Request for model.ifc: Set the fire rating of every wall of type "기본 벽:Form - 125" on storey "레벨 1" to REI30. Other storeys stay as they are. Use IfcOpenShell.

First a look at what the model holds.

```python
import ifcopenshell
import ifcopenshell.util.element

model = ifcopenshell.open("model.ifc")
print(model.schema)
storey = next(s for s in model.by_type("IfcBuildingStorey") if s.Name == "레벨 1")
walls = [e for e in ifcopenshell.util.element.get_decomposition(storey) if e.is_a("IfcWall")]
seen = {}
for e in walls:
    element_type = ifcopenshell.util.element.get_type(e)
    key = (element_type.Name if element_type != e and element_type else None, ifcopenshell.util.element.get_pset(e, "Pset_WallCommon", "FireRating"))
    seen[key] = seen.get(key, 0) + 1
for (name, value), count in sorted(seen.items(), key=str):
    print(count, "x", name, "|", value)
```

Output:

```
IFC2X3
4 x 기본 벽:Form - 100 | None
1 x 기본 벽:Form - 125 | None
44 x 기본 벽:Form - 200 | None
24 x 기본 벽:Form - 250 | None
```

```python
import ifcopenshell
import ifcopenshell.api.pset
import ifcopenshell.util.element

model = ifcopenshell.open("model.ifc")

storey = next(s for s in model.by_type("IfcBuildingStorey") if s.Name == "레벨 1")
walls = [e for e in ifcopenshell.util.element.get_decomposition(storey) if e.is_a("IfcWall")]

count = 0
for e in walls:
    element_type = ifcopenshell.util.element.get_type(e)
    if element_type in (None, e) or element_type.Name != "기본 벽:Form - 125":
        continue
    # add_pset returns the element's existing set when there is one.
    pset = ifcopenshell.api.pset.add_pset(model, product=e, name="Pset_WallCommon")
    ifcopenshell.api.pset.edit_pset(model, pset=pset, properties={"FireRating": "REI30"})
    count += 1

print(count, "walls updated")

model.write("model_rev.ifc")
```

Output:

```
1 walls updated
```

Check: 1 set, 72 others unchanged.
